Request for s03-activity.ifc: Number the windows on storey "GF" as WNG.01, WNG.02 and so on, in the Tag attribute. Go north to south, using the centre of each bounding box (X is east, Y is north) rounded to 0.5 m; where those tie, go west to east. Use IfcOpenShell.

First a look at what the model holds.

```python
import ifcopenshell
import ifcopenshell.util.element
import ifcopenshell.util.placement

model = ifcopenshell.open("s03-activity.ifc")
print(model.schema)
storey = next(s for s in model.by_type("IfcBuildingStorey") if s.Name == "GF")
windows = [e for e in ifcopenshell.util.element.get_decomposition(storey) if e.is_a("IfcWindow")]
for e in sorted(windows, key=lambda e: e.id()):
    origin = ifcopenshell.util.placement.get_local_placement(e.ObjectPlacement)[:3, 3]
    print(e.id(), e.Tag, e.Name, origin.round(2) + 0.0, sep=" | ")
```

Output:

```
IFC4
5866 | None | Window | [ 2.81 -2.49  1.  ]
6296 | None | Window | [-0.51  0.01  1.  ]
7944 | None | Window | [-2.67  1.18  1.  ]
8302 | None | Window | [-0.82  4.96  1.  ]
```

```python
import ifcopenshell
import ifcopenshell.geom
import ifcopenshell.util.element
import ifcopenshell.util.shape

model = ifcopenshell.open("s03-activity.ifc")
settings = ifcopenshell.geom.settings()
settings.set("use-world-coords", True)


def centre(element):
    shape = ifcopenshell.geom.create_shape(settings, element)
    return ifcopenshell.util.shape.get_bbox_centroid(shape.geometry)


storey = next(s for s in model.by_type("IfcBuildingStorey") if s.Name == "GF")
windows = [e for e in ifcopenshell.util.element.get_decomposition(storey) if e.is_a("IfcWindow")]

# Insertion points can sit at a corner or the storey origin, so sort by the geometry (in metres).
centres = {e: centre(e) for e in windows}
windows.sort(key=lambda e: (-round(centres[e][1] / 0.5), centres[e][0]))

for i, e in enumerate(windows, start=1):
    number = f"WNG.{i:02d}"
    e.Tag = number
    print(e.id(), number)

model.write("s03-activity_edited.ifc")
```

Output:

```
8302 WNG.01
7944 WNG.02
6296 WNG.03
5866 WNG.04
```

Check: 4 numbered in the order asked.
